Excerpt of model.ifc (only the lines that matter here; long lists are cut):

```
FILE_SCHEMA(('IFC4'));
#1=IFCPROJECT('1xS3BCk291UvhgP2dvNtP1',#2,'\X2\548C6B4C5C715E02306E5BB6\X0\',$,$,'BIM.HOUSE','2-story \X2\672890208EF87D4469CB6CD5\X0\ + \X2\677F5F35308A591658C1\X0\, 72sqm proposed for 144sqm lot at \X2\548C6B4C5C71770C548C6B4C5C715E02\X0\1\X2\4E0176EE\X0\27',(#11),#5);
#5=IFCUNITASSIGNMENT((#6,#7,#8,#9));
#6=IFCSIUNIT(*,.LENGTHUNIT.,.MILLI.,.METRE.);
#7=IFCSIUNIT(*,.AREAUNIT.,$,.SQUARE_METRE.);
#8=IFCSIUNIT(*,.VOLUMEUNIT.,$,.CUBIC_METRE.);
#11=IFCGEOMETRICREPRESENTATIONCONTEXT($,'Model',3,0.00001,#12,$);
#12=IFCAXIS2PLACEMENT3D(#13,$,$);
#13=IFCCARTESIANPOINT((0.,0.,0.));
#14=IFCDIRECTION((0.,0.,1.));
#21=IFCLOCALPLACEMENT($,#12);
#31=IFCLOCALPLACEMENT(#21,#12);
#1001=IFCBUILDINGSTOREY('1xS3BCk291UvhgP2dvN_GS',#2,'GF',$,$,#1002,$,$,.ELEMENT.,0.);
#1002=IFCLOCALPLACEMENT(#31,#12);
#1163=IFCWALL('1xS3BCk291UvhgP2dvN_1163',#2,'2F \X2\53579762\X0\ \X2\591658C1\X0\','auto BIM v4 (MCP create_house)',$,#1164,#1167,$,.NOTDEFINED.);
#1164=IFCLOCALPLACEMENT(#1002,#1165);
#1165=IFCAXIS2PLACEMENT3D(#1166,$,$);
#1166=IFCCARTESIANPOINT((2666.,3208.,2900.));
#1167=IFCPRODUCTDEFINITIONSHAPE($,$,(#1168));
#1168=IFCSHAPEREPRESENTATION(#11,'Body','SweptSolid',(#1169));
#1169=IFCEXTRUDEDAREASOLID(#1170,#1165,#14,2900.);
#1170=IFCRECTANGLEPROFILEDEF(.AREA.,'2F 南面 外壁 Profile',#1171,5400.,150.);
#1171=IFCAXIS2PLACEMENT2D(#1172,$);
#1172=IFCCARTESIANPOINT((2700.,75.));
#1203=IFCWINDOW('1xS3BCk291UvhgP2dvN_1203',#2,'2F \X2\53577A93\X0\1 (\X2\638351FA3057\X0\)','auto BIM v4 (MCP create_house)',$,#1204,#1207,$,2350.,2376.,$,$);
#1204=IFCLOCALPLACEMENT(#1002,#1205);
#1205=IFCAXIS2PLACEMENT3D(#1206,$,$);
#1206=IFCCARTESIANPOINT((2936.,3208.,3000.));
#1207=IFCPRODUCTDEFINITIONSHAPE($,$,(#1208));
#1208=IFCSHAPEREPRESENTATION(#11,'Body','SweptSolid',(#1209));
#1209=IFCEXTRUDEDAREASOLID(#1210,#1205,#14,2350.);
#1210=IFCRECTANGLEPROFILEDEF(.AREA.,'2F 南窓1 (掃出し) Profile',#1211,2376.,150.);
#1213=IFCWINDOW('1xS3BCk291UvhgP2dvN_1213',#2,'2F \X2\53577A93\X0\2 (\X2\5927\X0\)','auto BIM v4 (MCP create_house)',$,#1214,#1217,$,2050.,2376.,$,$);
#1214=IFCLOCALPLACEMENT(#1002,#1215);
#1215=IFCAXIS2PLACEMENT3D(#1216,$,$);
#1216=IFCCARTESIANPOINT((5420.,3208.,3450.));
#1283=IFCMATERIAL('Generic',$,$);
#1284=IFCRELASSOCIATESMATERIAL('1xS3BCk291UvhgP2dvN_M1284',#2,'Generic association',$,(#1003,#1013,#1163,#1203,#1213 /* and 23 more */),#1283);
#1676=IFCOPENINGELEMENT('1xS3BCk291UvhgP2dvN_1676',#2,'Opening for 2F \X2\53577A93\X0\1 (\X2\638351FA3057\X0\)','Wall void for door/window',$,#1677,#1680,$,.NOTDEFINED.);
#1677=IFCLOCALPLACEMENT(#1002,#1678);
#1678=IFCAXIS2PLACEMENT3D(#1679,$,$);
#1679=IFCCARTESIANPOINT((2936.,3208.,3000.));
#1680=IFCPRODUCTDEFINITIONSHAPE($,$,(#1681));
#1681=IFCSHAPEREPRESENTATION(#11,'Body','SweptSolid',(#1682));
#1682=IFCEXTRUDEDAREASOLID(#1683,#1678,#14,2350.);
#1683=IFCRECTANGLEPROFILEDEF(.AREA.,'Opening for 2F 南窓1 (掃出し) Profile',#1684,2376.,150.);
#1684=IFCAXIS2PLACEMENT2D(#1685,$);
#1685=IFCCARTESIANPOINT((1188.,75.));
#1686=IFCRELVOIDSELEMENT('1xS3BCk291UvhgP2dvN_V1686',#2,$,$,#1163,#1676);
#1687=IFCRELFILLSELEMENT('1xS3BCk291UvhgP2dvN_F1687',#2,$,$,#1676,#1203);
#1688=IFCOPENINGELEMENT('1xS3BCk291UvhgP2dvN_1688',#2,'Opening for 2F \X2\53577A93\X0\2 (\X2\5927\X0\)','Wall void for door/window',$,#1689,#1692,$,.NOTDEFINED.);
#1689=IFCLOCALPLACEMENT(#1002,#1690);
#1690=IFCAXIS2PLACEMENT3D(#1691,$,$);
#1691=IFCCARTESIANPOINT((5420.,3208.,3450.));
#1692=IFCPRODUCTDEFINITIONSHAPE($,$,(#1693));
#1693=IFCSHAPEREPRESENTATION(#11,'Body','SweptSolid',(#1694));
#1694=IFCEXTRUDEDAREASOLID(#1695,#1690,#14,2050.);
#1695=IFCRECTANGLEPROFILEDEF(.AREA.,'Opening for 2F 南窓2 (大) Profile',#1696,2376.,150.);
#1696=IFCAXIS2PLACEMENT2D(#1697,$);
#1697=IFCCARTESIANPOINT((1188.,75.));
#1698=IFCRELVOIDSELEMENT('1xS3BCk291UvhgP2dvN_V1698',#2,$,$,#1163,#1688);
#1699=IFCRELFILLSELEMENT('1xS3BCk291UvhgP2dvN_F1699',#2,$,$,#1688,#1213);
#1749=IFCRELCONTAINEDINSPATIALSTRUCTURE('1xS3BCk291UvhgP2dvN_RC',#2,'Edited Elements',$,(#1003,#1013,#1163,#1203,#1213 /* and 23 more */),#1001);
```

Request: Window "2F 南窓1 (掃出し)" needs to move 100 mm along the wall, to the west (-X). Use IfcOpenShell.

```python
import ifcopenshell
import ifcopenshell.api.geometry
import ifcopenshell.util.placement
import ifcopenshell.util.unit

model = ifcopenshell.open("model.ifc")
unit_scale = ifcopenshell.util.unit.calculate_unit_scale(model)

window = model.by_guid("1xS3BCk291UvhgP2dvN_1203")
opening = window.FillsVoids[0].RelatingOpeningElement
wall = opening.VoidsElements[0].RelatingBuildingElement

wall_matrix = ifcopenshell.util.placement.get_local_placement(wall.ObjectPlacement)
shift = wall_matrix[:3, 0] * -0.1 / unit_scale
before = ifcopenshell.util.placement.get_local_placement(window.ObjectPlacement)[:3, 3].copy()

# The window is not placed relative to its opening, so move both.
for product in (opening, window):
    matrix = ifcopenshell.util.placement.get_local_placement(product.ObjectPlacement)
    matrix[:3, 3] += shift
    ifcopenshell.api.geometry.edit_object_placement(model, product=product, matrix=matrix, is_si=False)

after = ifcopenshell.util.placement.get_local_placement(window.ObjectPlacement)[:3, 3]
print("window moved by", (after - before).round(3) + 0.0)

model.write("model_rev.ifc")
```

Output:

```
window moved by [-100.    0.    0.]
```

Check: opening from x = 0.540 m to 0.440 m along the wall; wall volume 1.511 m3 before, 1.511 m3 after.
